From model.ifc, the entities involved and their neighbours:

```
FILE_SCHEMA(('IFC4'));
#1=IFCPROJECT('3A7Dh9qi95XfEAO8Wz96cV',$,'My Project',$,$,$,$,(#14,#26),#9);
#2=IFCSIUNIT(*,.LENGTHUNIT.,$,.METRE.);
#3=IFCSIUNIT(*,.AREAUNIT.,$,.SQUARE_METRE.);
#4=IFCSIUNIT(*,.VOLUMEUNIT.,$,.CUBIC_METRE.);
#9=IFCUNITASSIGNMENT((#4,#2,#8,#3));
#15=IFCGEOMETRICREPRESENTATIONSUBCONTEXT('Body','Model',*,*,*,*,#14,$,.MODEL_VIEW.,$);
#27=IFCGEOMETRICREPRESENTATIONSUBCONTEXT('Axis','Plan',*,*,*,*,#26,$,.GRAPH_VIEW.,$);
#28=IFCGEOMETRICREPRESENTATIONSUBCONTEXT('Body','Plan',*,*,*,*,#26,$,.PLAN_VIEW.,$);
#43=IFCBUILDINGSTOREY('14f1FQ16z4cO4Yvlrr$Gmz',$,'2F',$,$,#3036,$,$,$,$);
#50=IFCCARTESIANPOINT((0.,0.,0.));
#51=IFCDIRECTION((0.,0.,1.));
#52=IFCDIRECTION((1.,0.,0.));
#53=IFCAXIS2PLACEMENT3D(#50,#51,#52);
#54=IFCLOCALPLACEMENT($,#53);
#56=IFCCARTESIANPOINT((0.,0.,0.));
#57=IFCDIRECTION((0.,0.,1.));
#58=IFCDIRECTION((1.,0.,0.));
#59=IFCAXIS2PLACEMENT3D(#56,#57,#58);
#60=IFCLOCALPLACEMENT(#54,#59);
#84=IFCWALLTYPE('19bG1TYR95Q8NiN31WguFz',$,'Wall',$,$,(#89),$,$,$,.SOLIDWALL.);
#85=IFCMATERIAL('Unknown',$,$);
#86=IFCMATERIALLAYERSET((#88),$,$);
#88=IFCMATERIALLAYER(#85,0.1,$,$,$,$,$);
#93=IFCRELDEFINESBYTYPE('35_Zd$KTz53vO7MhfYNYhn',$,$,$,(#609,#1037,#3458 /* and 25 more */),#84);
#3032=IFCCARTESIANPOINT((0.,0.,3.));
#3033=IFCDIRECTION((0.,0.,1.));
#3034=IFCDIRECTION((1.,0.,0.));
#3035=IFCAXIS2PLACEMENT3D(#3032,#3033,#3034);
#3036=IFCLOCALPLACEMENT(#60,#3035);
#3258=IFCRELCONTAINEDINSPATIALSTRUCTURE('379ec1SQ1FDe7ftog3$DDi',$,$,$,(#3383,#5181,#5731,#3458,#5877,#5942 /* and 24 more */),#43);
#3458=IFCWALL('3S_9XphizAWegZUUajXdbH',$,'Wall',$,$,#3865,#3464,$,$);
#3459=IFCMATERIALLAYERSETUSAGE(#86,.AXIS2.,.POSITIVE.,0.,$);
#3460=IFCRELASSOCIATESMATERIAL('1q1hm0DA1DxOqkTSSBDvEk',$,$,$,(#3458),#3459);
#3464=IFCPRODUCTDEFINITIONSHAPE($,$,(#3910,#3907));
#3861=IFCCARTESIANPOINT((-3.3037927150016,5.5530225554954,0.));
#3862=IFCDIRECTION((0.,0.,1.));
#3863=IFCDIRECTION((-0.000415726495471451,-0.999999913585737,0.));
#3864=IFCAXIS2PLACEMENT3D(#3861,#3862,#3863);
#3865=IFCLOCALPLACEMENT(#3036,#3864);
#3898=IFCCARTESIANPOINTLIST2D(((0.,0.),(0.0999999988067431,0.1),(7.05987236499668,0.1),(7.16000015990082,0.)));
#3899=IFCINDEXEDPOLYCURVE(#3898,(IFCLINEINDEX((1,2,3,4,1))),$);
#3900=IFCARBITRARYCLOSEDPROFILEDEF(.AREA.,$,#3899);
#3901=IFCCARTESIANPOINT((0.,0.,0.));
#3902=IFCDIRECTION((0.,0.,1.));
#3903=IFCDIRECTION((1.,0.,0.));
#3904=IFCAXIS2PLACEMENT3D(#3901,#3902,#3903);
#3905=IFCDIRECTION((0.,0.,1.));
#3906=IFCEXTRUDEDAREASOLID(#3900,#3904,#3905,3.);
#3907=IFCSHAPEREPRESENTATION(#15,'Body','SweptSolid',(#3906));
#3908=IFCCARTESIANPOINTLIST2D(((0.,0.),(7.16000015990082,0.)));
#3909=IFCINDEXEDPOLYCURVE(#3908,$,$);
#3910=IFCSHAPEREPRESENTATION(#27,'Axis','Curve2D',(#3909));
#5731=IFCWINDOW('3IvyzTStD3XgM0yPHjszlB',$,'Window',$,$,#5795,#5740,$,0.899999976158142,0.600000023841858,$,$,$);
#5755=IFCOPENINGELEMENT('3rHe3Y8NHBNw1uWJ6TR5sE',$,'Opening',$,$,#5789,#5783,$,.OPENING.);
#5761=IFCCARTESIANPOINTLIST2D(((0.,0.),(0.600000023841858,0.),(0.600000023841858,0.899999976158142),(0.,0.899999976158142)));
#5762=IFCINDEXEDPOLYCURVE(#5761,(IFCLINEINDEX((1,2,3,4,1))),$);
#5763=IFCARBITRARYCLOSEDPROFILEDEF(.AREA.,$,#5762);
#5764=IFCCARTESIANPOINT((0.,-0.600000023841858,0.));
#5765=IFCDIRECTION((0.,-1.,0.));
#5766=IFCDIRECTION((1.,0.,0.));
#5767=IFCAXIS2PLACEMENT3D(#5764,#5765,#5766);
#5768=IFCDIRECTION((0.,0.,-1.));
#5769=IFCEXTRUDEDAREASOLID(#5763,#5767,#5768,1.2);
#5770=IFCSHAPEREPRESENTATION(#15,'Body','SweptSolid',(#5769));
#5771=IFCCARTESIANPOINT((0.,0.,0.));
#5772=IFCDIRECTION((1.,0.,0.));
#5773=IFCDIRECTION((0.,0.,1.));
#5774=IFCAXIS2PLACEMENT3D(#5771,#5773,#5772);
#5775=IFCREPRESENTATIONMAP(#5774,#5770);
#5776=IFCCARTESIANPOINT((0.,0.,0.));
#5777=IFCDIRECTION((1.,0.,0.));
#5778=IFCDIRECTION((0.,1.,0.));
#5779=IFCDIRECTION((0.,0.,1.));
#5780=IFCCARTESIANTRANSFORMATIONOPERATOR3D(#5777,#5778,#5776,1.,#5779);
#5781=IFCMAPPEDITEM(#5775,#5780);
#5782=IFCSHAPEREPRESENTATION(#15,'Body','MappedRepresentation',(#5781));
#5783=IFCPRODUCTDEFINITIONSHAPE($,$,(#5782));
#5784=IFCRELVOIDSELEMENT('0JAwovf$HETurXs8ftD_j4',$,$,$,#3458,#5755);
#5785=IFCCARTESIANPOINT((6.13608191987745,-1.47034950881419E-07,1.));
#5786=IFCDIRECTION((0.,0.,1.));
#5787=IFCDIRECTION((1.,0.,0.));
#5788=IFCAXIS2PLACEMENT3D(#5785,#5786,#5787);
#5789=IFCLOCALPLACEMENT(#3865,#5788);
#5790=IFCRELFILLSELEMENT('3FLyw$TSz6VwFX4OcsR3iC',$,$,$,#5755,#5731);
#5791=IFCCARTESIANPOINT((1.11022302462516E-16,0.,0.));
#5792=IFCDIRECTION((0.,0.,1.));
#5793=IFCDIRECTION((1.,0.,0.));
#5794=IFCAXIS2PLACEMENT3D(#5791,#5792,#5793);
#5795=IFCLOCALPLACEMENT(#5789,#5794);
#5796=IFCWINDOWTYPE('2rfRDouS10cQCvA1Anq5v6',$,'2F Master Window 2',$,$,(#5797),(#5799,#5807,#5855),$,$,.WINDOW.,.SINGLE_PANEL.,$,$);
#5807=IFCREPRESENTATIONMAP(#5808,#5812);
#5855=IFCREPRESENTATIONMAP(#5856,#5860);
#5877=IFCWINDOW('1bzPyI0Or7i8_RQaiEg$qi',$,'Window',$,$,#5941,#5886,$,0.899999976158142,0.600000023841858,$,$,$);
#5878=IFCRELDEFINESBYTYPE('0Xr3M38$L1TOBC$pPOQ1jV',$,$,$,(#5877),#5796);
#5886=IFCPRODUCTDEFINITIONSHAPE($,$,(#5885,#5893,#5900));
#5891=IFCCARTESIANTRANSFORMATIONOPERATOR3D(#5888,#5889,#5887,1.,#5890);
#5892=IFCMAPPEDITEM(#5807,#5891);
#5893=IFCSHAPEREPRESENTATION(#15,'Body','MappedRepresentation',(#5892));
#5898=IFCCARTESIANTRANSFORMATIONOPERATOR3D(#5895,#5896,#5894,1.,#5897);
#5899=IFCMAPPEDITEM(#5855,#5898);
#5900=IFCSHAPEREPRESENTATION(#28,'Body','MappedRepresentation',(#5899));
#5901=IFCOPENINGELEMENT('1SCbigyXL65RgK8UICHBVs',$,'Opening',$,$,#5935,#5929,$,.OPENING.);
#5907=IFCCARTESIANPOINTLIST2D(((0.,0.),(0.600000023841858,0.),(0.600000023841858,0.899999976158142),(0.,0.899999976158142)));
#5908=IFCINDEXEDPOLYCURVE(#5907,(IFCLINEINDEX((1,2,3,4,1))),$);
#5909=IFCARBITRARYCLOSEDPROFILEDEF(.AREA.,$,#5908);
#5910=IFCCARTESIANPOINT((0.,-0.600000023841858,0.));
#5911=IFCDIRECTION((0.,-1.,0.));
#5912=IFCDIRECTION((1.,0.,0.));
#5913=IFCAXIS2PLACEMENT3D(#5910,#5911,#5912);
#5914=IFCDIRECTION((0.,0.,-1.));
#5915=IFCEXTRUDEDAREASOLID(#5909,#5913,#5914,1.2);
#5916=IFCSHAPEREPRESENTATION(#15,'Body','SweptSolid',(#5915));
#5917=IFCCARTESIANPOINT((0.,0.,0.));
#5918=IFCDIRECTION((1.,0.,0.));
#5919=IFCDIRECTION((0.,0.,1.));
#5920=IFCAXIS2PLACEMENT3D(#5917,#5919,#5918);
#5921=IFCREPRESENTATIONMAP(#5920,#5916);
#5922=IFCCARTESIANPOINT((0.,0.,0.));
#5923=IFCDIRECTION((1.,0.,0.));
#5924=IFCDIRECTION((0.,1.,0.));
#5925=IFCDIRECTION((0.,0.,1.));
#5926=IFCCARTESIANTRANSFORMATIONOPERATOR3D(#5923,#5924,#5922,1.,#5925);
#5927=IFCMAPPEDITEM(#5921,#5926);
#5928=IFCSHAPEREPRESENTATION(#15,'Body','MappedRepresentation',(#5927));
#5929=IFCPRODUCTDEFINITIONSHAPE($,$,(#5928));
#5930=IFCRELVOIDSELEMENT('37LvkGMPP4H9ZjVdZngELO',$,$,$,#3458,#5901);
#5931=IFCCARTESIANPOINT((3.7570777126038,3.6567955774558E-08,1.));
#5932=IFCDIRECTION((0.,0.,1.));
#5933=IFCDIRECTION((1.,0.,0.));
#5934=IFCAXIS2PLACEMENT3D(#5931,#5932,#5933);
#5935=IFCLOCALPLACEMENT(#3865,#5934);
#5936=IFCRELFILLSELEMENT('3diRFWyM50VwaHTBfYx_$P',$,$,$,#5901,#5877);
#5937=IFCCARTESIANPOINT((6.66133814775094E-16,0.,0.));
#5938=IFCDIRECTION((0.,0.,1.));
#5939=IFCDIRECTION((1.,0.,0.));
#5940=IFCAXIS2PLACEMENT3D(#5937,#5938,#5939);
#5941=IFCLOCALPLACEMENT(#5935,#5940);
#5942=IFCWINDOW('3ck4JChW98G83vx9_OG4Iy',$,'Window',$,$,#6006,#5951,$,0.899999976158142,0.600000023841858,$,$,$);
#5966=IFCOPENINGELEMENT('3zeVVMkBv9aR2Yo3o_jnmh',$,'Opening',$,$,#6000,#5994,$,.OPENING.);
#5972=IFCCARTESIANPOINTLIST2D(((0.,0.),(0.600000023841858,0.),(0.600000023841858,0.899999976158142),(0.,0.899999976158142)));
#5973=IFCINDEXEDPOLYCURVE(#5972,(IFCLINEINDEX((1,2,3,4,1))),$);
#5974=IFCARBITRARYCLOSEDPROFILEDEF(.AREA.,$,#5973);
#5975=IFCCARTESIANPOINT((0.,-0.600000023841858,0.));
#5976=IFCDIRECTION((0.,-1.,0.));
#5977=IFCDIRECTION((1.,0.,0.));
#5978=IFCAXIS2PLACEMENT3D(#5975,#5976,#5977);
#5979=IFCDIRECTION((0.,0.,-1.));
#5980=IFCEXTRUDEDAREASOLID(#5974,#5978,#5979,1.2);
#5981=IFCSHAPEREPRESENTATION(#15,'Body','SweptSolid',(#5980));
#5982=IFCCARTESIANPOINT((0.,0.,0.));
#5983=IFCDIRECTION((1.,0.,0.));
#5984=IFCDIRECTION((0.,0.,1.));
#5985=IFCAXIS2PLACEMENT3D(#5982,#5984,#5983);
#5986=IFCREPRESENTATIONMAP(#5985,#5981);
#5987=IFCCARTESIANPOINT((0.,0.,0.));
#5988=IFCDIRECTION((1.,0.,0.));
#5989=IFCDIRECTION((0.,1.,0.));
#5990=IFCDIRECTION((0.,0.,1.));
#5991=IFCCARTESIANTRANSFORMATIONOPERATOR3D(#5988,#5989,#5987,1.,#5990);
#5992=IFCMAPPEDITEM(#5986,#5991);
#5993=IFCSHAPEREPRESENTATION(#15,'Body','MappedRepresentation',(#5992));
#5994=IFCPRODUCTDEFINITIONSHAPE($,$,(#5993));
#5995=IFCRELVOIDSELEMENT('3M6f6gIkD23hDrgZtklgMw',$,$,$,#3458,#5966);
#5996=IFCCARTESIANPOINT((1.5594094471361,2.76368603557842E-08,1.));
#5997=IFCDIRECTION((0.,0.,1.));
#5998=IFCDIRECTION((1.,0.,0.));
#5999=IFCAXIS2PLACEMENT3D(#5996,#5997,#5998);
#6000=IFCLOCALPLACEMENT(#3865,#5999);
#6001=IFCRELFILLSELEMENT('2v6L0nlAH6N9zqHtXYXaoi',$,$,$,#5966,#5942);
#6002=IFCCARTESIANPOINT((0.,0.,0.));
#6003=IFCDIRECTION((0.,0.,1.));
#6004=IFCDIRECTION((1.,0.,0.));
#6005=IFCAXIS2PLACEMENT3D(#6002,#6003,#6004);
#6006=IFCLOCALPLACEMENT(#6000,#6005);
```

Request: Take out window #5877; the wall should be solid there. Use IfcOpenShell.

```python
import ifcopenshell
import ifcopenshell.api.feature
import ifcopenshell.api.root
import ifcopenshell.geom
import ifcopenshell.util.shape

model = ifcopenshell.open("model.ifc")
settings = ifcopenshell.geom.settings()


def volume(element):
    """Net volume in cubic metres, openings subtracted."""
    shape = ifcopenshell.geom.create_shape(settings, element)
    return ifcopenshell.util.shape.get_volume(shape.geometry)


window = model.by_guid("1bzPyI0Or7i8_RQaiEg$qi")
opening = window.FillsVoids[0].RelatingOpeningElement
wall = opening.VoidsElements[0].RelatingBuildingElement
before = volume(wall)

ifcopenshell.api.root.remove_product(model, product=window)
ifcopenshell.api.feature.remove_feature(model, feature=opening)

after = volume(wall)

print(f"wall volume {before:.3f} -> {after:.3f} m3")

model.write("model_rev.ifc")
```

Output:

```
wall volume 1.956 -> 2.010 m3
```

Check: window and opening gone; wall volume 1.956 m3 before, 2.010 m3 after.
